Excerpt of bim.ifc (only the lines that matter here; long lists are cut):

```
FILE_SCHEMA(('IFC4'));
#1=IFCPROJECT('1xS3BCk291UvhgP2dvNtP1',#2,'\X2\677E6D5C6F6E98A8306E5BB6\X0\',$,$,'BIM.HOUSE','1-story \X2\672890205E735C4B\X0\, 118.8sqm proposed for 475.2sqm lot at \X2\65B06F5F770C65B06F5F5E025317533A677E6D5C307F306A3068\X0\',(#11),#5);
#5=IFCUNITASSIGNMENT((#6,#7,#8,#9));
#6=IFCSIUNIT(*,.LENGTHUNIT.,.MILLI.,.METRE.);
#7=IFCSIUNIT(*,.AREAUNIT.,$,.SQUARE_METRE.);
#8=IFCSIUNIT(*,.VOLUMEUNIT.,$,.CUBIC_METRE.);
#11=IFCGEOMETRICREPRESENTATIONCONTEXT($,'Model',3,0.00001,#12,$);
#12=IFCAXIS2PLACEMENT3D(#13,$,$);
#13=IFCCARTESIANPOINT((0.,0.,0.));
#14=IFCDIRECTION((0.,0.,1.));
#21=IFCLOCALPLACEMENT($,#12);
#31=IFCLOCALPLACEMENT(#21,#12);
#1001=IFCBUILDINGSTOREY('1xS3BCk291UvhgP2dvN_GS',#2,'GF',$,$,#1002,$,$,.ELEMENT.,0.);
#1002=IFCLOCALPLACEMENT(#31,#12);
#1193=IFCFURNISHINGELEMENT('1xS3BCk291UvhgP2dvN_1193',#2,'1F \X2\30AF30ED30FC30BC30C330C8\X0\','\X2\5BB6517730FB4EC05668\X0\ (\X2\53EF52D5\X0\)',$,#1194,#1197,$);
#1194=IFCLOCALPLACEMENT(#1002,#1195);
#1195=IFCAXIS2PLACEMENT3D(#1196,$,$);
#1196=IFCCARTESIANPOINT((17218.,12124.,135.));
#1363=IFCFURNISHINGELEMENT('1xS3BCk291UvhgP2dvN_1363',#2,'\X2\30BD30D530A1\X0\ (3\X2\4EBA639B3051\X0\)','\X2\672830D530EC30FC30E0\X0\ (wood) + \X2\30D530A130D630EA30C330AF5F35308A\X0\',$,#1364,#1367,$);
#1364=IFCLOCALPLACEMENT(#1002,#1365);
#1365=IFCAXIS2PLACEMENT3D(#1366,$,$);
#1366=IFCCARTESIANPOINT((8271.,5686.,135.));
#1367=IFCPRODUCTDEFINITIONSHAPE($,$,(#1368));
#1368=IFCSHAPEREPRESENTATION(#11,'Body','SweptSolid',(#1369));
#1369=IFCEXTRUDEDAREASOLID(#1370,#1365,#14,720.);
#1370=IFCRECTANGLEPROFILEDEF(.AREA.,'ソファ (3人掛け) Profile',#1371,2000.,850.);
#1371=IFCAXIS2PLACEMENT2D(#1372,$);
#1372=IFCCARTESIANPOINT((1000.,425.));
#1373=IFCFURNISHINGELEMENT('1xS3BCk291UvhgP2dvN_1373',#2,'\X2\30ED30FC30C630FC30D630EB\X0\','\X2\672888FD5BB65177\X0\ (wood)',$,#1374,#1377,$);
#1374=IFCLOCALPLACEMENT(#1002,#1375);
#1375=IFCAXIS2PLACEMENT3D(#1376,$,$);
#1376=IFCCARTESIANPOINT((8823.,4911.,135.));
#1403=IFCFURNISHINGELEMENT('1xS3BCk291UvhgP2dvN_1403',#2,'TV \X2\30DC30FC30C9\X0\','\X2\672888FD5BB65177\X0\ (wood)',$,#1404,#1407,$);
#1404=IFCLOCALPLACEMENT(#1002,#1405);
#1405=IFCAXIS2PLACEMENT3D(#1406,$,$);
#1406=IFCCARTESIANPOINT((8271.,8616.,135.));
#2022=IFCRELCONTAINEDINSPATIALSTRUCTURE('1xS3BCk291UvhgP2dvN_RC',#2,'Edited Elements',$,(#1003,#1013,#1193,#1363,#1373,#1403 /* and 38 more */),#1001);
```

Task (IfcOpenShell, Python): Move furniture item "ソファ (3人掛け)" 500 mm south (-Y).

```python
import ifcopenshell
import ifcopenshell.api.geometry
import ifcopenshell.util.placement

model = ifcopenshell.open("bim.ifc")

item = model.by_id(1363)
matrix = ifcopenshell.util.placement.get_local_placement(item.ObjectPlacement)
matrix[1, 3] -= 500.0
ifcopenshell.api.geometry.edit_object_placement(model, product=item, matrix=matrix, is_si=False)

print(ifcopenshell.util.placement.get_local_placement(item.ObjectPlacement).round(3) + 0.0)

model.write("bim_v2.ifc")
```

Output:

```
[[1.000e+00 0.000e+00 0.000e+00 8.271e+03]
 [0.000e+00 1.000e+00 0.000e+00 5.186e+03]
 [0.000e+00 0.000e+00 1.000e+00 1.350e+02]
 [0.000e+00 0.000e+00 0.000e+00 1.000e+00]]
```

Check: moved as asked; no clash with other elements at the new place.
